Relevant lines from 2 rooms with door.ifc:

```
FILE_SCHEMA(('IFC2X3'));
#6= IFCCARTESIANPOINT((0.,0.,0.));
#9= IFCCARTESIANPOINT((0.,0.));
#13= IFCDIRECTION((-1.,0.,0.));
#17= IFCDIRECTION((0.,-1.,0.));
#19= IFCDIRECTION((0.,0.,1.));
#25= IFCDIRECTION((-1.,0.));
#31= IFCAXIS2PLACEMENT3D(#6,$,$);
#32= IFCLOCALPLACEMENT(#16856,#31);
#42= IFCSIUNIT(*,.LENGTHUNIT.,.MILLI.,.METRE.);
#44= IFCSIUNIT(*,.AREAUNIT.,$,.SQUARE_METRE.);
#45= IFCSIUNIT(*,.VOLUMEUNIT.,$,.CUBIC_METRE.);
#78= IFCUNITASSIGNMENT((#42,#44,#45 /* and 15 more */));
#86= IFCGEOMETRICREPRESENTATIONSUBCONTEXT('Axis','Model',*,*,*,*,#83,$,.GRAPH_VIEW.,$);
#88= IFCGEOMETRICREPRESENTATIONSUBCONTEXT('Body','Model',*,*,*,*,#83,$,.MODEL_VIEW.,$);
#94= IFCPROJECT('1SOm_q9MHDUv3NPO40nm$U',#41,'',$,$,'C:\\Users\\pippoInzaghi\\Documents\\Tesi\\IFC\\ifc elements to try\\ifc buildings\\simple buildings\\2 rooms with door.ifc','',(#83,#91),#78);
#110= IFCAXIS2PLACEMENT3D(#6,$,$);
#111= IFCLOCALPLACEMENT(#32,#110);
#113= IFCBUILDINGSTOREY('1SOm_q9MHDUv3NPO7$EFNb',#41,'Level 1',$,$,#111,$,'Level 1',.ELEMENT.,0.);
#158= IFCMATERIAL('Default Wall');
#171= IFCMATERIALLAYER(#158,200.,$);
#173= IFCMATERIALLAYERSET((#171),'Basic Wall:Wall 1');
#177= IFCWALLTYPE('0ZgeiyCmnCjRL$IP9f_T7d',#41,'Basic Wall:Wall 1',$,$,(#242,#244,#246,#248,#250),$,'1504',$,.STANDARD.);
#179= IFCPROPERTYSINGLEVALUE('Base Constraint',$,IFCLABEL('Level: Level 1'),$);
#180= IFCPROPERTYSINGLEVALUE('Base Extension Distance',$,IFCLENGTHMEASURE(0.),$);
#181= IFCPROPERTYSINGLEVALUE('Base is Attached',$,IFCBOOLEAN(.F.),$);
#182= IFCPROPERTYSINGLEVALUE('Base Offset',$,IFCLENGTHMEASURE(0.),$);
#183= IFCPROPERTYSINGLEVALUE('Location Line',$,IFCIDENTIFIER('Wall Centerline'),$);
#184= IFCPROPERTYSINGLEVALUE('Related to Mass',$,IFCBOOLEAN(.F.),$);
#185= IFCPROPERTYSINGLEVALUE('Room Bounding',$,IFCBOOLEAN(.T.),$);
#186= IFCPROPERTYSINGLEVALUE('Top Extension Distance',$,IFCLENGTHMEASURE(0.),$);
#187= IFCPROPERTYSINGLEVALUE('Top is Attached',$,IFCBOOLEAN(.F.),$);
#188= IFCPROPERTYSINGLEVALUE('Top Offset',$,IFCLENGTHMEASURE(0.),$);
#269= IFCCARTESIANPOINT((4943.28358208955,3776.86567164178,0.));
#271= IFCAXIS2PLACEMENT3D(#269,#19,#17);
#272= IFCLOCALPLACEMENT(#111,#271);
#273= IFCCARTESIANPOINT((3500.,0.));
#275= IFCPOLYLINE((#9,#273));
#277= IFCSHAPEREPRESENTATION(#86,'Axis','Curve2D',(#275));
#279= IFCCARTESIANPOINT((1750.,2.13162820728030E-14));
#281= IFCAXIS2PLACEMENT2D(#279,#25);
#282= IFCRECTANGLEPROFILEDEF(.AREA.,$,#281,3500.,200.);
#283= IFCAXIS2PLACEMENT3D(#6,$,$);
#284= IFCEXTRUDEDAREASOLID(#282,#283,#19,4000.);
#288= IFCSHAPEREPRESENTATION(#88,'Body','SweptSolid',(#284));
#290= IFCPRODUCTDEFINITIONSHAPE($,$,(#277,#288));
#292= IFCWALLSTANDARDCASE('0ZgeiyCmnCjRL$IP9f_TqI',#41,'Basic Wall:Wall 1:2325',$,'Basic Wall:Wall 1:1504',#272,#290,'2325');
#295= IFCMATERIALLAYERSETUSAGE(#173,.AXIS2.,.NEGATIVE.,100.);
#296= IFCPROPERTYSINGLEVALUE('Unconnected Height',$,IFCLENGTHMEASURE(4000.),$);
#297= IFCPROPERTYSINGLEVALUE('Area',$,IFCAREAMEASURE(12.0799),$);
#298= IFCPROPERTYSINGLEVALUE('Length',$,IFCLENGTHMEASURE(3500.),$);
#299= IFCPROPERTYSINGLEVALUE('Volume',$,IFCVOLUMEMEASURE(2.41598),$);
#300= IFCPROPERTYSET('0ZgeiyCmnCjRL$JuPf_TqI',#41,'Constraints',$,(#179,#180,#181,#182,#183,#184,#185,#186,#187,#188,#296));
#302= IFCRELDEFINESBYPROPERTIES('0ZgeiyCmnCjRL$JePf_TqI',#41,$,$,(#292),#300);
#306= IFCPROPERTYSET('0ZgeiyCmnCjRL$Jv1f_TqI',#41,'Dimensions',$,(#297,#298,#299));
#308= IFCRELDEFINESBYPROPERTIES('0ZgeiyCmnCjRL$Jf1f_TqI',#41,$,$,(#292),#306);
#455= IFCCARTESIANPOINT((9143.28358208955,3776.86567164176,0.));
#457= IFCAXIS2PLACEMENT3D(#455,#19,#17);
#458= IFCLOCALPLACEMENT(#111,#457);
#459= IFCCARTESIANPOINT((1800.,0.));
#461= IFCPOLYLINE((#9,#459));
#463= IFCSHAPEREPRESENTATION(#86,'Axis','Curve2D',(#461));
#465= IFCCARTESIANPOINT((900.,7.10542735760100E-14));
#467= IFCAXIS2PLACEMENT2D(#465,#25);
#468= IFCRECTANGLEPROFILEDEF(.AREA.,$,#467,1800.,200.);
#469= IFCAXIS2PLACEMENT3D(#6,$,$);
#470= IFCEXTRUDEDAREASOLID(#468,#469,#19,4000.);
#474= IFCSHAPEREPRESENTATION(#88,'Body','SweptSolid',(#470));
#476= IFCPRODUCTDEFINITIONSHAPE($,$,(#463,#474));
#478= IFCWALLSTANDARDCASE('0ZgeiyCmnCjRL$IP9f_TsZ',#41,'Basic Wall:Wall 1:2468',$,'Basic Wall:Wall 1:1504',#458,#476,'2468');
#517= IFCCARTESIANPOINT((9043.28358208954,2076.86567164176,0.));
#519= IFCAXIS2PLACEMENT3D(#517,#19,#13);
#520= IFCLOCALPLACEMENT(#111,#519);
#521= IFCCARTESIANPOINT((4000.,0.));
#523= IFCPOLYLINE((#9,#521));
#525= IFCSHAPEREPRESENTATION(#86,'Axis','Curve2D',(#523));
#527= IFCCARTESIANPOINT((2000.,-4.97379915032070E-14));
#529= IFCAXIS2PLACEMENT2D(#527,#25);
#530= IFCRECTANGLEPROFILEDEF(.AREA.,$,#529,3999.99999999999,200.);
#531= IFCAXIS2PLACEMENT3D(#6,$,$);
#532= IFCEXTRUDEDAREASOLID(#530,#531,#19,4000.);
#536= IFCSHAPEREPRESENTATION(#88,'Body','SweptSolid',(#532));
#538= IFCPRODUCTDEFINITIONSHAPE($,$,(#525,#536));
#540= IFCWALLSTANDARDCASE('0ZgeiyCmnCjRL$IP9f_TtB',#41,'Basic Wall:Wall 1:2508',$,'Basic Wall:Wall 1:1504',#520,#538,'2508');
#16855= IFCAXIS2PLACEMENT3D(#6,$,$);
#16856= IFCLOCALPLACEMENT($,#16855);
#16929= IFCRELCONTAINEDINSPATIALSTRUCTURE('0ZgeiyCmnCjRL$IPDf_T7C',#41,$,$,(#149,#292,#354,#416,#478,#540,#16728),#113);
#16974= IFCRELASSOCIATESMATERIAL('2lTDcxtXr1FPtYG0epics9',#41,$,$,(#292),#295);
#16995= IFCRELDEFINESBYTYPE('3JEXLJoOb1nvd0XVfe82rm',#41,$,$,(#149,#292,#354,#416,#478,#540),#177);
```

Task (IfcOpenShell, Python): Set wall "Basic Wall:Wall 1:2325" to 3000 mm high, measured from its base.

```python
import ifcopenshell
import ifcopenshell.api.pset
import ifcopenshell.geom
import ifcopenshell.util.element
import ifcopenshell.util.representation
import ifcopenshell.util.shape
import ifcopenshell.util.unit

model = ifcopenshell.open("2 rooms with door.ifc")
unit_scale = ifcopenshell.util.unit.calculate_unit_scale(model)
area_scale = ifcopenshell.util.unit.calculate_unit_scale(model, "AREAUNIT")
volume_scale = ifcopenshell.util.unit.calculate_unit_scale(model, "VOLUMEUNIT")
settings = ifcopenshell.geom.settings()


def volume(element):
    """Net volume in cubic metres, openings subtracted."""
    shape = ifcopenshell.geom.create_shape(settings, element)
    return ifcopenshell.util.shape.get_volume(shape.geometry)


wall = model.by_guid("0ZgeiyCmnCjRL$IP9f_TqI")
before = volume(wall)

body = ifcopenshell.util.representation.get_representation(wall, "Model", "Body")
solid = body.Items[0]
old_height = solid.Depth
solid.Depth = 3 / unit_scale
after = volume(wall)
thickness = 0.2  # wall thickness in metres

# Update the stored height, areas and volumes.
pset = model.by_id(ifcopenshell.util.element.get_pset(wall, "Constraints", should_inherit=False)["id"])
ifcopenshell.api.pset.edit_pset(model, pset=pset, properties={
    "Unconnected Height": model.create_entity("IfcLengthMeasure", solid.Depth),
})
pset = model.by_id(ifcopenshell.util.element.get_pset(wall, "Dimensions", should_inherit=False)["id"])
ifcopenshell.api.pset.edit_pset(model, pset=pset, properties={
    "Area": model.create_entity("IfcAreaMeasure", after / thickness / area_scale),
    "Volume": model.create_entity("IfcVolumeMeasure", after / volume_scale),
})

print(f"height {old_height:g} -> {solid.Depth:g}, volume {before:.3f} -> {after:.3f} m3")

model.write("2 rooms with door_rev.ifc")
```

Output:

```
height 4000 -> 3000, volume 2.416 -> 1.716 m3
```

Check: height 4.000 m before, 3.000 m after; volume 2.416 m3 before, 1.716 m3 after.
